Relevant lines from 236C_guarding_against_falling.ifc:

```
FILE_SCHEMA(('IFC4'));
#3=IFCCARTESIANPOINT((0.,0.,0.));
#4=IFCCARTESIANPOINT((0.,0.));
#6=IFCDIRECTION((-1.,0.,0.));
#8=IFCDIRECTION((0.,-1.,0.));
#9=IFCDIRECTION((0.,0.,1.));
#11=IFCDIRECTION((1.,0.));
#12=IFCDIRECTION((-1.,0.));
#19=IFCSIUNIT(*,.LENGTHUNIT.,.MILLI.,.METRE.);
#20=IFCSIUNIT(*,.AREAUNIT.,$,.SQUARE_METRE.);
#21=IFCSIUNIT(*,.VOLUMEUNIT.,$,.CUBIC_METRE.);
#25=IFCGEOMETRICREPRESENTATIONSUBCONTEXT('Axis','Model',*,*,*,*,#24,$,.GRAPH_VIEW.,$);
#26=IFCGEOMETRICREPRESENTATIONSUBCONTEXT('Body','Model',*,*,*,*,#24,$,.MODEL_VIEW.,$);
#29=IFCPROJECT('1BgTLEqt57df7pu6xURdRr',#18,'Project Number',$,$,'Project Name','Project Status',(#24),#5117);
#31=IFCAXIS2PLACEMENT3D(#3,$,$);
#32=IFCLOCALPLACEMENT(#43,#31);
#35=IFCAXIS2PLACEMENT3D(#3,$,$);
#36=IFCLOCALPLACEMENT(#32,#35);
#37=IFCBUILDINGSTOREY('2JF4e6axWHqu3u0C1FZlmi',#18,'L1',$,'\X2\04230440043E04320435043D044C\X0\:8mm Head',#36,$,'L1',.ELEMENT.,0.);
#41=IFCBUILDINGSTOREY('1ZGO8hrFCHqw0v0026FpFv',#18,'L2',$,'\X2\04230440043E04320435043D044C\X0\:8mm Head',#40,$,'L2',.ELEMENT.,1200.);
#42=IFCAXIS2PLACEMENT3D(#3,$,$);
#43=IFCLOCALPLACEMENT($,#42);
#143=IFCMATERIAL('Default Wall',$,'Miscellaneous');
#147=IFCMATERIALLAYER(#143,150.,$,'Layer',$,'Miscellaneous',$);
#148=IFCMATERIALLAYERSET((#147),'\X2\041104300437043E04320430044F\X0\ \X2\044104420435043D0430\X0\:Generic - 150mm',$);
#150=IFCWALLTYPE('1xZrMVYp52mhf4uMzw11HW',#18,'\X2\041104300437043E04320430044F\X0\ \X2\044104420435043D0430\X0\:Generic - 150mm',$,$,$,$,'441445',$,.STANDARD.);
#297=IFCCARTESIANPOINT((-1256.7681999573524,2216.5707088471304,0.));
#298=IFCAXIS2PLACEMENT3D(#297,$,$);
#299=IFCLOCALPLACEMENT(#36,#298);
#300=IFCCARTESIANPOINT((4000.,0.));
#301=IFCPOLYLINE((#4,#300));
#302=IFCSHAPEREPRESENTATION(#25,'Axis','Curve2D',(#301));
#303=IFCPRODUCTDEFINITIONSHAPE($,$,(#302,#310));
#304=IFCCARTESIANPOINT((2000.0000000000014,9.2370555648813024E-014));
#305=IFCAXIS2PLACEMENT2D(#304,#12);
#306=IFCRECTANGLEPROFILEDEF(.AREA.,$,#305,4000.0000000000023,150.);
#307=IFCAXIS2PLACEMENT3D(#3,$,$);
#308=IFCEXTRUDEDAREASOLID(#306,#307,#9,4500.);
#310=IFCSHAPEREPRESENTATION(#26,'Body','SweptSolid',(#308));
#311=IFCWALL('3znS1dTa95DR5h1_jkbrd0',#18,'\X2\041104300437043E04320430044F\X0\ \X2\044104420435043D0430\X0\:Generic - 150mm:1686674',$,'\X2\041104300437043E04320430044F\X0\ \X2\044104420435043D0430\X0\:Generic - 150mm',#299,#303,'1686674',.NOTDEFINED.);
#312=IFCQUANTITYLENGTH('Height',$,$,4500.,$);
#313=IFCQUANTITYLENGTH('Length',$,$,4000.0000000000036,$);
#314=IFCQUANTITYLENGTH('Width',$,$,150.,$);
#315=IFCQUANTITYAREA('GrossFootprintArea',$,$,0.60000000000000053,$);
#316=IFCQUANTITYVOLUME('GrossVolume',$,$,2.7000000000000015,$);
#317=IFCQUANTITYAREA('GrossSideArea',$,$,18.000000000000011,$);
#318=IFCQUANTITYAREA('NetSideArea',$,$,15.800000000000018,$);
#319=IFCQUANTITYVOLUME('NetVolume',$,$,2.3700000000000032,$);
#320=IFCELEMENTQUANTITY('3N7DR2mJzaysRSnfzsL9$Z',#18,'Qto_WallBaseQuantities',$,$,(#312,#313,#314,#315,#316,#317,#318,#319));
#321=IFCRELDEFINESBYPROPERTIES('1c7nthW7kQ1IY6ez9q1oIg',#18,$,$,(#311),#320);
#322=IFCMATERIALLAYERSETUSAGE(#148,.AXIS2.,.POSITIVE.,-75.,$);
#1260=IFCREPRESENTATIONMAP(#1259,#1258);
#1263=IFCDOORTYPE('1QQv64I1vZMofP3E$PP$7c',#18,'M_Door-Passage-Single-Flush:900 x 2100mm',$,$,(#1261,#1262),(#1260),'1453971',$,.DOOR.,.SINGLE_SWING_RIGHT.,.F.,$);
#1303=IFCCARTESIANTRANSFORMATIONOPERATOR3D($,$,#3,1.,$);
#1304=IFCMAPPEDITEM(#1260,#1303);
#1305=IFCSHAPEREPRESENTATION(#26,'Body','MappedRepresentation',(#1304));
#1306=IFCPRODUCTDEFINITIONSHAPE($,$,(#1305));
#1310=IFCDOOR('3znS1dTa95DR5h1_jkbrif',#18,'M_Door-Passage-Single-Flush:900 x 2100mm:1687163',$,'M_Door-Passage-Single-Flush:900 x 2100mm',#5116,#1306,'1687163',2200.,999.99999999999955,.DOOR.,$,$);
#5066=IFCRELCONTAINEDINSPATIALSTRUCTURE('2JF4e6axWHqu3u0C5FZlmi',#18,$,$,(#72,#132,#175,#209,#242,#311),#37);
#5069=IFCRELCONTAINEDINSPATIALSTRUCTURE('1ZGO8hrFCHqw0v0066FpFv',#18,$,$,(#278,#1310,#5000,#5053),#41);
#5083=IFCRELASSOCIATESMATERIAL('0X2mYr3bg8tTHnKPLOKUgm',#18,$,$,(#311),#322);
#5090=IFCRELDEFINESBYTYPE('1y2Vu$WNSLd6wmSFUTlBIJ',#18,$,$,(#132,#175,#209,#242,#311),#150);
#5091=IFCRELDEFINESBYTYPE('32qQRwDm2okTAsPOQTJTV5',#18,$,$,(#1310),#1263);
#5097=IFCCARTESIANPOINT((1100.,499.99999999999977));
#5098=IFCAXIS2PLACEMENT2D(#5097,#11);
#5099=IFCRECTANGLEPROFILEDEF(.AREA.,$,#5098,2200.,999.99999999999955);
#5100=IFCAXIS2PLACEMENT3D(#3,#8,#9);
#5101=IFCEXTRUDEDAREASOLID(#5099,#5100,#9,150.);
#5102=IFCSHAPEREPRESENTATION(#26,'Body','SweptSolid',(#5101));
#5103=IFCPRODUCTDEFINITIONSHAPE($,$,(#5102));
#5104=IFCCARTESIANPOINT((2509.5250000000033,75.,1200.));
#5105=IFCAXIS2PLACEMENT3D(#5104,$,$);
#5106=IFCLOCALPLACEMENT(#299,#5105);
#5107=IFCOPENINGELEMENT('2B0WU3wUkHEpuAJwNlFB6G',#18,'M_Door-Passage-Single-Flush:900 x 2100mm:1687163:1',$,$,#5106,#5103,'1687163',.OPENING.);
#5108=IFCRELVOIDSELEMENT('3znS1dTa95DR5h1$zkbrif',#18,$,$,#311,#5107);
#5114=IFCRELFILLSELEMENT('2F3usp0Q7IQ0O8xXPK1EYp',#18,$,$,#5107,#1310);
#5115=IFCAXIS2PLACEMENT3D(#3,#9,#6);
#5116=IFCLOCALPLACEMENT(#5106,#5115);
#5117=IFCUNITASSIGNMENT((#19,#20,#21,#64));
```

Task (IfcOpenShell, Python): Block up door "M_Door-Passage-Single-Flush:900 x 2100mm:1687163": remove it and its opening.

```python
import ifcopenshell
import ifcopenshell.api.feature
import ifcopenshell.api.pset
import ifcopenshell.api.root
import ifcopenshell.geom
import ifcopenshell.util.element
import ifcopenshell.util.shape
import ifcopenshell.util.unit

model = ifcopenshell.open("236C_guarding_against_falling.ifc")
area_scale = ifcopenshell.util.unit.calculate_unit_scale(model, "AREAUNIT")
volume_scale = ifcopenshell.util.unit.calculate_unit_scale(model, "VOLUMEUNIT")
settings = ifcopenshell.geom.settings()


def volume(element):
    """Net volume in cubic metres, openings subtracted."""
    shape = ifcopenshell.geom.create_shape(settings, element)
    return ifcopenshell.util.shape.get_volume(shape.geometry)


door = model.by_guid("3znS1dTa95DR5h1_jkbrif")
opening = door.FillsVoids[0].RelatingOpeningElement
wall = opening.VoidsElements[0].RelatingBuildingElement
before = volume(wall)

ifcopenshell.api.root.remove_product(model, product=door)
ifcopenshell.api.feature.remove_feature(model, feature=opening)

after = volume(wall)
thickness = 0.15  # wall thickness in metres

# Update the wall's stored quantities.
qto = model.by_id(ifcopenshell.util.element.get_pset(wall, "Qto_WallBaseQuantities", should_inherit=False)["id"])
ifcopenshell.api.pset.edit_qto(model, qto=qto, properties={
    "NetSideArea": after / thickness / area_scale,
    "NetVolume": after / volume_scale,
})

print(f"wall volume {before:.3f} -> {after:.3f} m3")

model.write("236C_guarding_against_falling_edited.ifc")
```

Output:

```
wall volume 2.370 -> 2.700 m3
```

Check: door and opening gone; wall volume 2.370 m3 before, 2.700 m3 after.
